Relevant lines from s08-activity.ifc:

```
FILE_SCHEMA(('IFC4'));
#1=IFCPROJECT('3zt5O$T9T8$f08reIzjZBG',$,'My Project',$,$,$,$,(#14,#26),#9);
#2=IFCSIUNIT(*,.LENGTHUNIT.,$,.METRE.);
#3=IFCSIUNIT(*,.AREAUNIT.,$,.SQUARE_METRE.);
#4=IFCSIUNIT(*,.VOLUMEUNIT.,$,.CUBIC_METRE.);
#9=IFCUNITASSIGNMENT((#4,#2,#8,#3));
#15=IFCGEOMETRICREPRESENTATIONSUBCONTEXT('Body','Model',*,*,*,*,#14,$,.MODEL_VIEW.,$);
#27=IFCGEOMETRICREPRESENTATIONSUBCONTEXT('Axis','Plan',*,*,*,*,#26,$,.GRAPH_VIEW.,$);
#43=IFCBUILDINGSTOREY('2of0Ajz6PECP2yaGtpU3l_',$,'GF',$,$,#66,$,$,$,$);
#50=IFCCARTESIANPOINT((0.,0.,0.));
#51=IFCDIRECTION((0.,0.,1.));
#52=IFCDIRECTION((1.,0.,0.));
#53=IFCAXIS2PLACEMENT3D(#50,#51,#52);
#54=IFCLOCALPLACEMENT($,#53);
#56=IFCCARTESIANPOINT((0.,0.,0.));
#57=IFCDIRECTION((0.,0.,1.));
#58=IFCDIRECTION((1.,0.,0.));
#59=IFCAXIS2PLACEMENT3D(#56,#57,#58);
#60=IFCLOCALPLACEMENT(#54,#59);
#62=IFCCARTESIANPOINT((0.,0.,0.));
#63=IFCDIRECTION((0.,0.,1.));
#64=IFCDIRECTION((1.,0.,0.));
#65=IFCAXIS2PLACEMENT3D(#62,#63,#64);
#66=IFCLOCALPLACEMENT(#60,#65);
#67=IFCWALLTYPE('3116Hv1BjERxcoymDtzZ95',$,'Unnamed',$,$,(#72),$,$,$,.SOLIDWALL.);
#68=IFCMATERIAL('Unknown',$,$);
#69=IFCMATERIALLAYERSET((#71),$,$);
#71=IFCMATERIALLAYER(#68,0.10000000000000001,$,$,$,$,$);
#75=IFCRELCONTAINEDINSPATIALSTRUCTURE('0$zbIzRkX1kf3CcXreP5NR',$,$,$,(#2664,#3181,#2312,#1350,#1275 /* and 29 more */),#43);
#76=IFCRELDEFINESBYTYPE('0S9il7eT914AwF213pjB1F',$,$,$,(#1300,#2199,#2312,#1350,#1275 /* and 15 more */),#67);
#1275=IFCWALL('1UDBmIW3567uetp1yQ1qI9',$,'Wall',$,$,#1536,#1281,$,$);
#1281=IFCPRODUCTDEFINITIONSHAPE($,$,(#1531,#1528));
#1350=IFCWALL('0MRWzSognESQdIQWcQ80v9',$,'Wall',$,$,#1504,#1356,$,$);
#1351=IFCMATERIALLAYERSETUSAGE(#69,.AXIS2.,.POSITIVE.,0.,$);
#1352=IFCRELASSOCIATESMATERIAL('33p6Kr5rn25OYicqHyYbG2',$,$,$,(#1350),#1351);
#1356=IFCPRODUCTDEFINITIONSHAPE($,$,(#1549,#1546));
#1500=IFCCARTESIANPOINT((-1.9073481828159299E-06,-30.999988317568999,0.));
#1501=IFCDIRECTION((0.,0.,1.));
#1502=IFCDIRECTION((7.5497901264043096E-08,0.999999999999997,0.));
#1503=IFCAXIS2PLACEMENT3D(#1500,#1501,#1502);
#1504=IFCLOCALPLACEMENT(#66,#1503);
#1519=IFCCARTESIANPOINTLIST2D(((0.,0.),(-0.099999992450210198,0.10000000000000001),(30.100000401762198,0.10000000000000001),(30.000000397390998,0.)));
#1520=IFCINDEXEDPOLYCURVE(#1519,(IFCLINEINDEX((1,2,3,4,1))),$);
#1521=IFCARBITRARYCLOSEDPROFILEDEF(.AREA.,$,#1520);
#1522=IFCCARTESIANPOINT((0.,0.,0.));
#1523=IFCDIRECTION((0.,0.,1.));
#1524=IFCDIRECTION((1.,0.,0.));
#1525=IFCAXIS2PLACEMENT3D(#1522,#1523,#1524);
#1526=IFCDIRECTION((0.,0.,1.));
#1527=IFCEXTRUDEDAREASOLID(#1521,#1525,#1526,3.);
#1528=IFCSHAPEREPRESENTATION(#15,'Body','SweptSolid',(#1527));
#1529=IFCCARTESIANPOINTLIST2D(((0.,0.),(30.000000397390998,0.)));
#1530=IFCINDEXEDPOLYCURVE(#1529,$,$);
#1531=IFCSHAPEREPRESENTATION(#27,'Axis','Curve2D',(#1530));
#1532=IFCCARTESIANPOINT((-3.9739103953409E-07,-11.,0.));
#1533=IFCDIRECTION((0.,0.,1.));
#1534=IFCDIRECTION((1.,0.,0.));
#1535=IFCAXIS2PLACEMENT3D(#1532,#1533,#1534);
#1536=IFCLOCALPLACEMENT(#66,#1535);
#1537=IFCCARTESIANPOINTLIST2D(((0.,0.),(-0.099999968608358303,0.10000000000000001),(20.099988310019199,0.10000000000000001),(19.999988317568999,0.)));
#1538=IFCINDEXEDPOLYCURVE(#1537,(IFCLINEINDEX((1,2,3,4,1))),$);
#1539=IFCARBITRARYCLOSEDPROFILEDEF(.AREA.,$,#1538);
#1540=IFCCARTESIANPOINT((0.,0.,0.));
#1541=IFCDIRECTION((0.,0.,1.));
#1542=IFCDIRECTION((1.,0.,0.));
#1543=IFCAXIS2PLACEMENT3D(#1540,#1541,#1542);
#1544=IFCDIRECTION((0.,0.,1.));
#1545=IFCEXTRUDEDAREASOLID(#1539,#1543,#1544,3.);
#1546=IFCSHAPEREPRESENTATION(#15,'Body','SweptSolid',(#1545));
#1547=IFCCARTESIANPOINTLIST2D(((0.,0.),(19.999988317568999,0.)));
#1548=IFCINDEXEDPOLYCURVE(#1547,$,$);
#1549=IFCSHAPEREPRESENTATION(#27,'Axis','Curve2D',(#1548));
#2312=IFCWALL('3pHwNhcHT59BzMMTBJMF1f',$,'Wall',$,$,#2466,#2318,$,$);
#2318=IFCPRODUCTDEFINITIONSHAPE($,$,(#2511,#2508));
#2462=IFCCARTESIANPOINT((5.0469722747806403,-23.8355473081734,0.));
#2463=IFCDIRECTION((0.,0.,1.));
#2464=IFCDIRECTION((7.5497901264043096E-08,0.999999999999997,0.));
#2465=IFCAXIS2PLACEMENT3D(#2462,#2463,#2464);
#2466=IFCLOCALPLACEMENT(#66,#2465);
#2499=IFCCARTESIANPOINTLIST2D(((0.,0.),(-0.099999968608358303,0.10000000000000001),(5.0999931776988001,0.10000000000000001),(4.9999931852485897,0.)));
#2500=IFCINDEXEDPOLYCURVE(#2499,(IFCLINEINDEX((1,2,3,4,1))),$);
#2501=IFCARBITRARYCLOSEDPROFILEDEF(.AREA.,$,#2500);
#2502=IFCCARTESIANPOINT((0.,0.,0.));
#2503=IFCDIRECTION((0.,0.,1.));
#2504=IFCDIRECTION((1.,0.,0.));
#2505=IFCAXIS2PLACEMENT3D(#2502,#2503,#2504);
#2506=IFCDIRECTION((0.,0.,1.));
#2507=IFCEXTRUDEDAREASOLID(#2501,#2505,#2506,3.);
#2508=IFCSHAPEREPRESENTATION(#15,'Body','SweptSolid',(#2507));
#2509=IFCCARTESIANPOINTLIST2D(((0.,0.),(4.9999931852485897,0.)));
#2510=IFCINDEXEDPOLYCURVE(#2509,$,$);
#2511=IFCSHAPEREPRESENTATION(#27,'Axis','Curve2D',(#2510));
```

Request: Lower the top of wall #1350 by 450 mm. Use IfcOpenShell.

```python
import ifcopenshell
import ifcopenshell.geom
import ifcopenshell.util.representation
import ifcopenshell.util.shape

model = ifcopenshell.open("s08-activity.ifc")
settings = ifcopenshell.geom.settings()


def volume(element):
    """Net volume in cubic metres, openings subtracted."""
    shape = ifcopenshell.geom.create_shape(settings, element)
    return ifcopenshell.util.shape.get_volume(shape.geometry)


wall = model.by_guid("0MRWzSognESQdIQWcQ80v9")
before = volume(wall)

body = ifcopenshell.util.representation.get_representation(wall, "Model", "Body")
solid = body.Items[0]
old_height = solid.Depth
solid.Depth -= 0.45
after = volume(wall)

print(f"height {old_height:g} -> {solid.Depth:g}, volume {before:.3f} -> {after:.3f} m3")

model.write("s08-activity_rev.ifc")
```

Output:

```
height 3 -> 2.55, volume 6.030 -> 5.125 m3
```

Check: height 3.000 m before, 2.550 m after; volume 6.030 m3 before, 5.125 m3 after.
